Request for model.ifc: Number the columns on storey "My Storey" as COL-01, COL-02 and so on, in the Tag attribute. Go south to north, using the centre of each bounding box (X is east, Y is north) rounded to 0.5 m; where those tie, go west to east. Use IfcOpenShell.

First a look at what the model holds.

```python
import ifcopenshell
import ifcopenshell.util.element
import ifcopenshell.util.placement

model = ifcopenshell.open("model.ifc")
print(model.schema)
storey = next(s for s in model.by_type("IfcBuildingStorey") if s.Name == "My Storey")
columns = [e for e in ifcopenshell.util.element.get_decomposition(storey) if e.is_a("IfcColumn")]
for e in sorted(columns, key=lambda e: e.id()):
    origin = ifcopenshell.util.placement.get_local_placement(e.ObjectPlacement)[:3, 3]
    print(e.id(), e.Tag, e.Name, origin.round(2) + 0.0, sep=" | ")
```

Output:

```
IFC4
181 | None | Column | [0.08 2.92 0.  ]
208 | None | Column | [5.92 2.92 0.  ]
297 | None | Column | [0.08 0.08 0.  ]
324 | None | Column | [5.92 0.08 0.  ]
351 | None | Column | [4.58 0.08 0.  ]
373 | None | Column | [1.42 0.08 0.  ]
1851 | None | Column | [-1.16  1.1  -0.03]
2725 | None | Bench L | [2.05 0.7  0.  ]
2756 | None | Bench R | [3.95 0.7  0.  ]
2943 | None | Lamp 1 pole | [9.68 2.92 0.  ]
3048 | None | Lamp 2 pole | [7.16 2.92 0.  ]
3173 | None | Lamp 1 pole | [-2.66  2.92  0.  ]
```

```python
import ifcopenshell
import ifcopenshell.geom
import ifcopenshell.util.element
import ifcopenshell.util.shape

model = ifcopenshell.open("model.ifc")
settings = ifcopenshell.geom.settings()
settings.set("use-world-coords", True)


def centre(element):
    shape = ifcopenshell.geom.create_shape(settings, element)
    return ifcopenshell.util.shape.get_bbox_centroid(shape.geometry)


storey = next(s for s in model.by_type("IfcBuildingStorey") if s.Name == "My Storey")
columns = [e for e in ifcopenshell.util.element.get_decomposition(storey) if e.is_a("IfcColumn")]

# Insertion points can sit at a corner or the storey origin, so sort by the geometry (in metres).
centres = {e: centre(e) for e in columns}
columns.sort(key=lambda e: (round(centres[e][1] / 0.5), centres[e][0]))

for i, e in enumerate(columns, start=1):
    number = f"COL-{i:02d}"
    e.Tag = number
    print(e.id(), number)

model.write("model_updated.ifc")
```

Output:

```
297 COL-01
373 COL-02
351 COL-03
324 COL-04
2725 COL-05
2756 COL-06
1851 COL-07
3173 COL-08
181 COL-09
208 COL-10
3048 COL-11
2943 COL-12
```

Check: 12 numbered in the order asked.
